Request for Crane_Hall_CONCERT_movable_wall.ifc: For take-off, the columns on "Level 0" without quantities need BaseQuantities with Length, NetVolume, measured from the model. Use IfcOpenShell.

First a look at what the model holds.

```python
import ifcopenshell
import ifcopenshell.util.element
import ifcopenshell.util.unit

model = ifcopenshell.open("Crane_Hall_CONCERT_movable_wall.ifc")
print(model.schema)
for unit_type in ("LENGTHUNIT", "AREAUNIT", "VOLUMEUNIT"):
    print(unit_type, ifcopenshell.util.unit.calculate_unit_scale(model, unit_type))
storey = next(s for s in model.by_type("IfcBuildingStorey") if s.Name == "Level 0")
columns = [e for e in ifcopenshell.util.element.get_decomposition(storey) if e.is_a("IfcColumn")]
for e in sorted(columns, key=lambda e: e.id()):
    print(e.id(), e.is_a(), e.Name, list(ifcopenshell.util.element.get_psets(e, qtos_only=True)), sep=" | ")
```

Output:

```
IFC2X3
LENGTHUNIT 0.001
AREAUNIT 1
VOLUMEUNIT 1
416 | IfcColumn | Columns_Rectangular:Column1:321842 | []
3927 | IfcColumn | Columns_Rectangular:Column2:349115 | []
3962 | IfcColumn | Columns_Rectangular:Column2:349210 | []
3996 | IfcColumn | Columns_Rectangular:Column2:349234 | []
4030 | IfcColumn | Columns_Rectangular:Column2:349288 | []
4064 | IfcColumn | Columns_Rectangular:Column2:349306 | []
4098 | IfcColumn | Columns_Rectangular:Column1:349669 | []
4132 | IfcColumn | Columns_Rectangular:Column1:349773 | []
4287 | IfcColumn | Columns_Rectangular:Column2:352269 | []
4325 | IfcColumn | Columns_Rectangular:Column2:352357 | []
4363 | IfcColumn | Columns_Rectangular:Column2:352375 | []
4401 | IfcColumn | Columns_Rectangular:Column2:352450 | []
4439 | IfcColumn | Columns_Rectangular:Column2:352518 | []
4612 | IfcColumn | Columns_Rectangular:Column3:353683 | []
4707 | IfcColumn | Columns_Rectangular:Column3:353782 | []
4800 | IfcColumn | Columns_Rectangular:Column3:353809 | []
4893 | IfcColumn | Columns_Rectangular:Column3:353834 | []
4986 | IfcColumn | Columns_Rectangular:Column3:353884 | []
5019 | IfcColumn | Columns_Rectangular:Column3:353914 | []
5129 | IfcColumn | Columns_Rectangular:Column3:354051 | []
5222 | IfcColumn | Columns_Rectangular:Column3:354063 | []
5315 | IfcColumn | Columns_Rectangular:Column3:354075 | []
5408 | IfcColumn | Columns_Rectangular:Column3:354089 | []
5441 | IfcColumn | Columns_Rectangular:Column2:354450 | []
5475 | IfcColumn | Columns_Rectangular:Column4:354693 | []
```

```python
import ifcopenshell
import ifcopenshell.api.pset
import ifcopenshell.geom
import ifcopenshell.util.element
import ifcopenshell.util.shape
import ifcopenshell.util.unit

model = ifcopenshell.open("Crane_Hall_CONCERT_movable_wall.ifc")
unit_scale = ifcopenshell.util.unit.calculate_unit_scale(model)
volume_scale = ifcopenshell.util.unit.calculate_unit_scale(model, "VOLUMEUNIT")
settings = ifcopenshell.geom.settings()

storey = next(s for s in model.by_type("IfcBuildingStorey") if s.Name == "Level 0")
columns = [e for e in ifcopenshell.util.element.get_decomposition(storey) if e.is_a("IfcColumn")]

for e in sorted(columns, key=lambda e: e.id()):
    if ifcopenshell.util.element.get_psets(e, qtos_only=True, should_inherit=False):
        continue
    # Geometry comes back in metres, in the element's own axes.
    shape = ifcopenshell.geom.create_shape(settings, e)
    values = {
        "Length": ifcopenshell.util.shape.get_z(shape.geometry) / unit_scale,
        "NetVolume": ifcopenshell.util.shape.get_volume(shape.geometry) / volume_scale,
    }
    qto = ifcopenshell.api.pset.add_qto(model, product=e, name="BaseQuantities")
    ifcopenshell.api.pset.edit_qto(model, qto=qto, properties=values)
    print(e.id(), {k: round(v, 3) for k, v in values.items()})

model.write("Crane_Hall_CONCERT_movable_wall_v2.ifc")
```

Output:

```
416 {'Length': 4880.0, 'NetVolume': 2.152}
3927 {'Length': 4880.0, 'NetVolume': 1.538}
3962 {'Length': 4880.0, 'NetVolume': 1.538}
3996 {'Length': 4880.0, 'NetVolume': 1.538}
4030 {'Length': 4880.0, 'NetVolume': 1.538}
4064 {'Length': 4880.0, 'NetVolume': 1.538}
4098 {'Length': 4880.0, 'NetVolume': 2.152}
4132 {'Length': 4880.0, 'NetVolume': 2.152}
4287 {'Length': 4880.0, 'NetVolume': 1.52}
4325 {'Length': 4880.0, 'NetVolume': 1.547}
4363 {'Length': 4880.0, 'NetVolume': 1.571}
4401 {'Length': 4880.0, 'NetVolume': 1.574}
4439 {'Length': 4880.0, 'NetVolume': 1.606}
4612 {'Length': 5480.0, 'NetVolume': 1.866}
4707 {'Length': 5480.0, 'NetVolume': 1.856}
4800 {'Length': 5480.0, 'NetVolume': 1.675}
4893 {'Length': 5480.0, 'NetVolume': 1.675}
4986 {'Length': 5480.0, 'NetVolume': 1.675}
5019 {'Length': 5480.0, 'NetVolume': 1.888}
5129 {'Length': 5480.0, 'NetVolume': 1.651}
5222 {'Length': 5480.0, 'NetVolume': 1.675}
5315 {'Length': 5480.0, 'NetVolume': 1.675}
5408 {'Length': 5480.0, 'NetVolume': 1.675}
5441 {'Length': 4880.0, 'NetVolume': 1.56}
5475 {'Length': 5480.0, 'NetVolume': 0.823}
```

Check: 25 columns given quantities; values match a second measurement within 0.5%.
